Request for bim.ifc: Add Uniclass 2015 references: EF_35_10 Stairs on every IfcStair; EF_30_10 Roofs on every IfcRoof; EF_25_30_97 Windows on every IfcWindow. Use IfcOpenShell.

First a look at what the model holds.

```python
import ifcopenshell

model = ifcopenshell.open("bim.ifc")
print(model.schema)
print("classifications:", [c.Name for c in model.by_type("IfcClassification")])
for ifc_class in ("IfcDoor", "IfcRoof", "IfcStair", "IfcWall", "IfcWindow"):
    print(ifc_class, len(model.by_type(ifc_class)))
```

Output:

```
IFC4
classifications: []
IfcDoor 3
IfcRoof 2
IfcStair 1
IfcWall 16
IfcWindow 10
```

```python
import ifcopenshell
import ifcopenshell.api.classification

model = ifcopenshell.open("bim.ifc")

system = ifcopenshell.api.classification.add_classification(model, classification="Uniclass 2015")

codes = {
    "IfcStair": ("EF_35_10", "Stairs"),
    "IfcRoof": ("EF_30_10", "Roofs"),
    "IfcWindow": ("EF_25_30_97", "Windows"),
}
for ifc_class, (code, name) in codes.items():
    products = model.by_type(ifc_class)
    ifcopenshell.api.classification.add_reference(
        model, products=products, classification=system, identification=code, name=name
    )
    print(code, len(products))

model.write("bim_v2.ifc")
```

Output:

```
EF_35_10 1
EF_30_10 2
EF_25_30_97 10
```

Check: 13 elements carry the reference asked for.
